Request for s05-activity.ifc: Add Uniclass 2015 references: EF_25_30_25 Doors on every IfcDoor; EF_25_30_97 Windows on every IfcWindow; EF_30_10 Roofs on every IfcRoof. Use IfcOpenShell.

First a look at what the model holds.

```python
import ifcopenshell

model = ifcopenshell.open("s05-activity.ifc")
print(model.schema)
print("classifications:", [c.Name for c in model.by_type("IfcClassification")])
for ifc_class in ("IfcDoor", "IfcRoof", "IfcStair", "IfcWall", "IfcWindow"):
    print(ifc_class, len(model.by_type(ifc_class)))
```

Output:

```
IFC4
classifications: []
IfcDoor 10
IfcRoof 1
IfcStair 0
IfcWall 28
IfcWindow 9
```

```python
import ifcopenshell
import ifcopenshell.api.classification

model = ifcopenshell.open("s05-activity.ifc")

system = ifcopenshell.api.classification.add_classification(model, classification="Uniclass 2015")

codes = {
    "IfcDoor": ("EF_25_30_25", "Doors"),
    "IfcWindow": ("EF_25_30_97", "Windows"),
    "IfcRoof": ("EF_30_10", "Roofs"),
}
for ifc_class, (code, name) in codes.items():
    products = model.by_type(ifc_class)
    ifcopenshell.api.classification.add_reference(
        model, products=products, classification=system, identification=code, name=name
    )
    print(code, len(products))

model.write("s05-activity_v2.ifc")
```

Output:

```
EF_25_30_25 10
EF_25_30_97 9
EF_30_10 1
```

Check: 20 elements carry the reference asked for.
